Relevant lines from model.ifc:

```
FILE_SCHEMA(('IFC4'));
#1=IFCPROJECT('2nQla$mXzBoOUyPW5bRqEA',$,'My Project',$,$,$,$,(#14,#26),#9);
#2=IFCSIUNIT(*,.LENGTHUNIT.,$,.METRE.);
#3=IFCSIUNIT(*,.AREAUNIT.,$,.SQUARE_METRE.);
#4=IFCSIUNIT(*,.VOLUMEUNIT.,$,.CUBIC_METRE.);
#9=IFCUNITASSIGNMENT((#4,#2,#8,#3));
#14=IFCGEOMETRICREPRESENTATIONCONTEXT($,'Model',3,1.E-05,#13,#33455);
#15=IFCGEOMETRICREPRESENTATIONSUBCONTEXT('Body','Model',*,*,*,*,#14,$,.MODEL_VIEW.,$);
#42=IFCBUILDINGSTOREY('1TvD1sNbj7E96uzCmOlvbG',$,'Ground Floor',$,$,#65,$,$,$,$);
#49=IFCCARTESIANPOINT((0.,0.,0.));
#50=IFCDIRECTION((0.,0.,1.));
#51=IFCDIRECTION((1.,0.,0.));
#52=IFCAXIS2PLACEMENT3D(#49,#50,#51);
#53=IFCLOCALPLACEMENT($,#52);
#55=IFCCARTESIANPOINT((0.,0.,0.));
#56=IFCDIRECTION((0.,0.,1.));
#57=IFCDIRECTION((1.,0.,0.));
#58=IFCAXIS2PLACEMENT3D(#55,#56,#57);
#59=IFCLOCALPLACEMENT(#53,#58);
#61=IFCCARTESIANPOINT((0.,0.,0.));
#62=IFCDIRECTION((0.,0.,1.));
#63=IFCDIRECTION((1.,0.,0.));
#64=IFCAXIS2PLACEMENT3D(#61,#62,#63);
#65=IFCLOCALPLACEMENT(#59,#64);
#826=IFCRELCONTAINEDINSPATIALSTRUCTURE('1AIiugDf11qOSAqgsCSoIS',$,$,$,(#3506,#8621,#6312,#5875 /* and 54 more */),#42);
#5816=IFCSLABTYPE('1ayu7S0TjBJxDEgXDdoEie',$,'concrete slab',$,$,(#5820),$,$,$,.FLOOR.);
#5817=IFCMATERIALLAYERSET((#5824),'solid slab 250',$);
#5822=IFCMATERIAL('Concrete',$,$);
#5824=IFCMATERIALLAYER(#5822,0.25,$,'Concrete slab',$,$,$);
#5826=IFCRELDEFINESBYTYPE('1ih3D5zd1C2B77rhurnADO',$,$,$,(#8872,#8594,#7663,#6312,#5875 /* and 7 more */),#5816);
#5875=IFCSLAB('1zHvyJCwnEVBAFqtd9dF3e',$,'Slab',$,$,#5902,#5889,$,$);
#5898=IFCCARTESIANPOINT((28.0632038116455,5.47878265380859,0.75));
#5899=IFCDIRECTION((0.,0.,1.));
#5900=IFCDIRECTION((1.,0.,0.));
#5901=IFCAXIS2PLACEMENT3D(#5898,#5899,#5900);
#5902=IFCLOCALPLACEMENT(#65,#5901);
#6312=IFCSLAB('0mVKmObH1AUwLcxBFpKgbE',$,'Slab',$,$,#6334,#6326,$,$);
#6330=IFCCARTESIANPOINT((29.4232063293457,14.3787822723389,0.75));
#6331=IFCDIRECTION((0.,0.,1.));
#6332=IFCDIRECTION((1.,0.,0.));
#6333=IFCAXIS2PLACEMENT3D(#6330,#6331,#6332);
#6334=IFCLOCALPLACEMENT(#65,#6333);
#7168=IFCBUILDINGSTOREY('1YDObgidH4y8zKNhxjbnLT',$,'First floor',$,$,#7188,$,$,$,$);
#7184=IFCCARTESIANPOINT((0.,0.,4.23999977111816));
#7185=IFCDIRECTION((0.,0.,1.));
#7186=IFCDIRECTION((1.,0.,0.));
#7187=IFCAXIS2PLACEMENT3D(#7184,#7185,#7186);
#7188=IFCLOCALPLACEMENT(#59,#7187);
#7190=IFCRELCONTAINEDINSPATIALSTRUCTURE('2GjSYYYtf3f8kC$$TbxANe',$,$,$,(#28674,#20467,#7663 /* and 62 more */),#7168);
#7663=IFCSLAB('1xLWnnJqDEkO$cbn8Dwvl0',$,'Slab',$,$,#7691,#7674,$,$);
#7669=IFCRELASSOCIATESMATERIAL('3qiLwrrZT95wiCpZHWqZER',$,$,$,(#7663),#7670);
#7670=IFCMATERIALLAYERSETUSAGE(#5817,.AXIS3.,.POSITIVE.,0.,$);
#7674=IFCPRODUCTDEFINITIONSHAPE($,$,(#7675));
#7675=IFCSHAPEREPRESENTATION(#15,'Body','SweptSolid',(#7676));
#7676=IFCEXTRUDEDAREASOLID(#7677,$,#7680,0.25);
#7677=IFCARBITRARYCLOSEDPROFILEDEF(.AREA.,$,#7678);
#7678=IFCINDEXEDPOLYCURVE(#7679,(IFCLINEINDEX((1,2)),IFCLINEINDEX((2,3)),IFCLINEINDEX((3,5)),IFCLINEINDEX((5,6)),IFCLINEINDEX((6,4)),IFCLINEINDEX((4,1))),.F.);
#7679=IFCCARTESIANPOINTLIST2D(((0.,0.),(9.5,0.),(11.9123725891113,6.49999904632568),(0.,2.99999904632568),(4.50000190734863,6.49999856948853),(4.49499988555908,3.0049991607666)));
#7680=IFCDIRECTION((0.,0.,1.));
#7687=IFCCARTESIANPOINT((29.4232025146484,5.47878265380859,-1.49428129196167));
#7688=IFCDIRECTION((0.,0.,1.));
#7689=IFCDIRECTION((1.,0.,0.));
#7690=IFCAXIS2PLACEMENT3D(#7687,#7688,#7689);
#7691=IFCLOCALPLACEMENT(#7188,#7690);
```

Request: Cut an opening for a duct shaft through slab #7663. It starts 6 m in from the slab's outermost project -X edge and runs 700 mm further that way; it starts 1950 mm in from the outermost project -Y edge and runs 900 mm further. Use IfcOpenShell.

```python
import numpy as np
import ifcopenshell
import ifcopenshell.api.feature
import ifcopenshell.api.geometry
import ifcopenshell.api.root
import ifcopenshell.geom
import ifcopenshell.util.placement
import ifcopenshell.util.representation
import ifcopenshell.util.shape
import ifcopenshell.util.unit

model = ifcopenshell.open("model.ifc")
unit_scale = ifcopenshell.util.unit.calculate_unit_scale(model)
settings = ifcopenshell.geom.settings()


def volume(element):
    """Net volume in cubic metres, openings subtracted."""
    shape = ifcopenshell.geom.create_shape(settings, element)
    return ifcopenshell.util.shape.get_volume(shape.geometry)


slab = model.by_guid("1xLWnnJqDEkO$cbn8Dwvl0")
before = volume(slab)

# Extent in the slab's own axes, in metres. The edges named are its -X and -Y sides.
slab_shape = ifcopenshell.geom.create_shape(settings, slab)
vertices = ifcopenshell.util.shape.get_vertices(slab_shape.geometry)
x_min, y_min, bottom = vertices.min(axis=0)
top = vertices[:, 2].max()

opening = ifcopenshell.api.root.create_entity(model, ifc_class="IfcOpeningElement", name="Duct shaft opening", predefined_type="OPENING")
context = ifcopenshell.util.representation.get_context(model, "Model", "Body", "MODEL_VIEW")
width, depth = 0.7, 0.9
outline = [(0.0, 0.0), (width, 0.0), (width, depth), (0.0, depth), (0.0, 0.0)]
# Overshoot both faces by 50 mm so the cut is clean.
shape = ifcopenshell.api.geometry.add_slab_representation(
    model, context=context, depth=top - bottom + 0.1, polyline=outline
)
ifcopenshell.api.geometry.assign_representation(model, product=opening, representation=shape)

matrix = ifcopenshell.util.placement.get_local_placement(slab.ObjectPlacement)
matrix[:, 3] = matrix @ np.append(np.array([x_min + 6, y_min + 1.95, bottom - 0.05]) / unit_scale, 1.0)
ifcopenshell.api.geometry.edit_object_placement(model, product=opening, matrix=matrix, is_si=False)
ifcopenshell.api.feature.add_feature(model, feature=opening, element=slab)

after = volume(slab)

print(f"slab volume {before:.3f} -> {after:.3f} m3")

model.write("model_rev.ifc")
```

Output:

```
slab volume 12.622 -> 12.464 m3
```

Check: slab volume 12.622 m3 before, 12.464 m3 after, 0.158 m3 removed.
